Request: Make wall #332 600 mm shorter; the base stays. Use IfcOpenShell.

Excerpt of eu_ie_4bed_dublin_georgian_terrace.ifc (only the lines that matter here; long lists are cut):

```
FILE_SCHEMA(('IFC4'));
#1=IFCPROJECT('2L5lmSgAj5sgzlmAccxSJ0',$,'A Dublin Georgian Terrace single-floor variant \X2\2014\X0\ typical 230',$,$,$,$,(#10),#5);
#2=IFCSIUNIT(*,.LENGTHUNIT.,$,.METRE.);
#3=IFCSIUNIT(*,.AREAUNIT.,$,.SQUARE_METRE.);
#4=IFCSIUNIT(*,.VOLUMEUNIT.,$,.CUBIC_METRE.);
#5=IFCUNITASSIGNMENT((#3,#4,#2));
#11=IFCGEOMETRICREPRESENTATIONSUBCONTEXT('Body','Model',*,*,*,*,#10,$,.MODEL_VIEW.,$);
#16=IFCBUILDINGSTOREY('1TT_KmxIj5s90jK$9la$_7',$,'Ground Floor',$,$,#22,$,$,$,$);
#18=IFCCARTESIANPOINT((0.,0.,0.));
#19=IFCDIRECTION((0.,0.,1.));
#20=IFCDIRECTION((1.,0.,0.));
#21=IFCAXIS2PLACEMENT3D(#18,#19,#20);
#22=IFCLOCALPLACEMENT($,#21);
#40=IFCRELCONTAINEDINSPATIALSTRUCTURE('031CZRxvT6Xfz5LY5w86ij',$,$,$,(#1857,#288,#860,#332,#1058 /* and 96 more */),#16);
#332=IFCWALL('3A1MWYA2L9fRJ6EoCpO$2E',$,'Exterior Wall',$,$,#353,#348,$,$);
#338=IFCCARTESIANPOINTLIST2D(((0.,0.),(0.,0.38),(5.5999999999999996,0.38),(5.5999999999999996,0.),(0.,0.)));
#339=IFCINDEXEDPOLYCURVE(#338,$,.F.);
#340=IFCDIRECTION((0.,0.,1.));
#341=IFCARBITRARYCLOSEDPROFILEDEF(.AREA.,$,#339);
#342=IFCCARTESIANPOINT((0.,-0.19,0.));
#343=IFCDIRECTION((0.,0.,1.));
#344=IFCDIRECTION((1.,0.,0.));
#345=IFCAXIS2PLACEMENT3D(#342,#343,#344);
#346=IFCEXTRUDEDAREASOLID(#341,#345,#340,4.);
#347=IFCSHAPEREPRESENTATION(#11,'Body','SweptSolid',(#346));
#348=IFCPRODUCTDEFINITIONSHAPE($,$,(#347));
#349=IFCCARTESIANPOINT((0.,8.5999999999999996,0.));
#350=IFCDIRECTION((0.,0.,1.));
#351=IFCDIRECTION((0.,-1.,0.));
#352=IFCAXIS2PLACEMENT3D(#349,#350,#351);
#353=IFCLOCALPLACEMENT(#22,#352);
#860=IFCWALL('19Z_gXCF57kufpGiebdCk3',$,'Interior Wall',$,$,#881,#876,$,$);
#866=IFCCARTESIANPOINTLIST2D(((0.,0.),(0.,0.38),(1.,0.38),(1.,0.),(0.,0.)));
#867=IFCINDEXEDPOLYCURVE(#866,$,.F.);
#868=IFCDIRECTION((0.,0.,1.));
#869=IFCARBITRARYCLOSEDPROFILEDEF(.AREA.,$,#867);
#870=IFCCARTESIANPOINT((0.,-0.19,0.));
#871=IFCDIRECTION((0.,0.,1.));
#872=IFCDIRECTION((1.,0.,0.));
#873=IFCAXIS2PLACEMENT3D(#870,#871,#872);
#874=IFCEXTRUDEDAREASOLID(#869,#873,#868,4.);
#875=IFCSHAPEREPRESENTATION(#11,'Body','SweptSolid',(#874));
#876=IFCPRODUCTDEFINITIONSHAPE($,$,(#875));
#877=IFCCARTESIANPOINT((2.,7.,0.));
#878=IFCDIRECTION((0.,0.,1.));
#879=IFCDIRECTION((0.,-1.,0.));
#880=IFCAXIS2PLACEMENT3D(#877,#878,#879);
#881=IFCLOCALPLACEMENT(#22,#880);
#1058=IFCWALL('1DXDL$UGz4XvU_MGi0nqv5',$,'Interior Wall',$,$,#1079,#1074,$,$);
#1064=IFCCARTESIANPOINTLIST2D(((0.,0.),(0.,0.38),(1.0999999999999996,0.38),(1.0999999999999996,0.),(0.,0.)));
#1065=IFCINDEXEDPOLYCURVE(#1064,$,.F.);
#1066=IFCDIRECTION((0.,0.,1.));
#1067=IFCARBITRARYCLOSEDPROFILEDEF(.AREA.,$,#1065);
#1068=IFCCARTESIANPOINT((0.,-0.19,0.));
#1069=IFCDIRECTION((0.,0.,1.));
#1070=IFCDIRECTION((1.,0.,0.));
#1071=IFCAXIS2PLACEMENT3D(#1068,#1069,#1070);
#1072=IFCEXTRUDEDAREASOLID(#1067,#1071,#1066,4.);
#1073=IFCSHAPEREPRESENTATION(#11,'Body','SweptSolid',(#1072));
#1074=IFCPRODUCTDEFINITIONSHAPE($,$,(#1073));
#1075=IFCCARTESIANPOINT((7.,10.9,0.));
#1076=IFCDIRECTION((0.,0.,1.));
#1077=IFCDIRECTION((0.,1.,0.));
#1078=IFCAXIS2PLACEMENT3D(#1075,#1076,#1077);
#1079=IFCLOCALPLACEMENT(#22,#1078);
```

```python
import ifcopenshell
import ifcopenshell.geom
import ifcopenshell.util.representation
import ifcopenshell.util.shape
import ifcopenshell.util.unit

model = ifcopenshell.open("eu_ie_4bed_dublin_georgian_terrace.ifc")
unit_scale = ifcopenshell.util.unit.calculate_unit_scale(model)
settings = ifcopenshell.geom.settings()


def volume(element):
    """Net volume in cubic metres, openings subtracted."""
    shape = ifcopenshell.geom.create_shape(settings, element)
    return ifcopenshell.util.shape.get_volume(shape.geometry)


wall = model.by_id(332)
before = volume(wall)

body = ifcopenshell.util.representation.get_representation(wall, "Model", "Body")
solid = body.Items[0]
old_height = solid.Depth
solid.Depth -= 0.6 / unit_scale
after = volume(wall)

print(f"height {old_height:g} -> {solid.Depth:g}, volume {before:.3f} -> {after:.3f} m3")

model.write("eu_ie_4bed_dublin_georgian_terrace_v2.ifc")
```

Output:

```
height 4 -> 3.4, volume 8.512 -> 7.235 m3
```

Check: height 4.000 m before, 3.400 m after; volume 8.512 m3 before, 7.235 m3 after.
